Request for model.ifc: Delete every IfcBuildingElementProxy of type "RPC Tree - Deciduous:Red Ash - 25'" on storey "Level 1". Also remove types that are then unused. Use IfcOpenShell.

First a look at what the model holds.

```python
import ifcopenshell
import ifcopenshell.util.element

model = ifcopenshell.open("model.ifc")
print(model.schema)
storey = next(s for s in model.by_type("IfcBuildingStorey") if s.Name == "Level 1")
proxies = [e for e in ifcopenshell.util.element.get_decomposition(storey) if e.is_a("IfcBuildingElementProxy")]
seen = {}
for e in proxies:
    element_type = ifcopenshell.util.element.get_type(e)
    name = element_type.Name if element_type not in (None, e) else None
    seen[name] = seen.get(name, 0) + 1
for name, count in sorted(seen.items(), key=str):
    print(count, "x", name)
```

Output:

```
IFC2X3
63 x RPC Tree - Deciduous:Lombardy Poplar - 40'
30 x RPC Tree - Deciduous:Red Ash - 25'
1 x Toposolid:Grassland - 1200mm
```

```python
import ifcopenshell
import ifcopenshell.api.root
import ifcopenshell.util.element

model = ifcopenshell.open("model.ifc")

storey = next(s for s in model.by_type("IfcBuildingStorey") if s.Name == "Level 1")
proxies = [e for e in ifcopenshell.util.element.get_decomposition(storey) if e.is_a("IfcBuildingElementProxy")]
targets = [e for e in proxies if (t := ifcopenshell.util.element.get_type(e)) not in (None, e) and t.Name == "RPC Tree - Deciduous:Red Ash - 25'"]
types = {ifcopenshell.util.element.get_type(e) for e in targets} - {None, *targets}

for e in targets:
    ifcopenshell.api.root.remove_product(model, product=e)
print(len(targets), "removed")

unused = [t for t in types if not ifcopenshell.util.element.get_types(t)]
for t in unused:
    ifcopenshell.api.root.remove_product(model, product=t)
print(len(unused), "unused types removed")

model.write("model_updated.ifc")
```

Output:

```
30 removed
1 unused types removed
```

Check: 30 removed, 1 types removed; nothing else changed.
